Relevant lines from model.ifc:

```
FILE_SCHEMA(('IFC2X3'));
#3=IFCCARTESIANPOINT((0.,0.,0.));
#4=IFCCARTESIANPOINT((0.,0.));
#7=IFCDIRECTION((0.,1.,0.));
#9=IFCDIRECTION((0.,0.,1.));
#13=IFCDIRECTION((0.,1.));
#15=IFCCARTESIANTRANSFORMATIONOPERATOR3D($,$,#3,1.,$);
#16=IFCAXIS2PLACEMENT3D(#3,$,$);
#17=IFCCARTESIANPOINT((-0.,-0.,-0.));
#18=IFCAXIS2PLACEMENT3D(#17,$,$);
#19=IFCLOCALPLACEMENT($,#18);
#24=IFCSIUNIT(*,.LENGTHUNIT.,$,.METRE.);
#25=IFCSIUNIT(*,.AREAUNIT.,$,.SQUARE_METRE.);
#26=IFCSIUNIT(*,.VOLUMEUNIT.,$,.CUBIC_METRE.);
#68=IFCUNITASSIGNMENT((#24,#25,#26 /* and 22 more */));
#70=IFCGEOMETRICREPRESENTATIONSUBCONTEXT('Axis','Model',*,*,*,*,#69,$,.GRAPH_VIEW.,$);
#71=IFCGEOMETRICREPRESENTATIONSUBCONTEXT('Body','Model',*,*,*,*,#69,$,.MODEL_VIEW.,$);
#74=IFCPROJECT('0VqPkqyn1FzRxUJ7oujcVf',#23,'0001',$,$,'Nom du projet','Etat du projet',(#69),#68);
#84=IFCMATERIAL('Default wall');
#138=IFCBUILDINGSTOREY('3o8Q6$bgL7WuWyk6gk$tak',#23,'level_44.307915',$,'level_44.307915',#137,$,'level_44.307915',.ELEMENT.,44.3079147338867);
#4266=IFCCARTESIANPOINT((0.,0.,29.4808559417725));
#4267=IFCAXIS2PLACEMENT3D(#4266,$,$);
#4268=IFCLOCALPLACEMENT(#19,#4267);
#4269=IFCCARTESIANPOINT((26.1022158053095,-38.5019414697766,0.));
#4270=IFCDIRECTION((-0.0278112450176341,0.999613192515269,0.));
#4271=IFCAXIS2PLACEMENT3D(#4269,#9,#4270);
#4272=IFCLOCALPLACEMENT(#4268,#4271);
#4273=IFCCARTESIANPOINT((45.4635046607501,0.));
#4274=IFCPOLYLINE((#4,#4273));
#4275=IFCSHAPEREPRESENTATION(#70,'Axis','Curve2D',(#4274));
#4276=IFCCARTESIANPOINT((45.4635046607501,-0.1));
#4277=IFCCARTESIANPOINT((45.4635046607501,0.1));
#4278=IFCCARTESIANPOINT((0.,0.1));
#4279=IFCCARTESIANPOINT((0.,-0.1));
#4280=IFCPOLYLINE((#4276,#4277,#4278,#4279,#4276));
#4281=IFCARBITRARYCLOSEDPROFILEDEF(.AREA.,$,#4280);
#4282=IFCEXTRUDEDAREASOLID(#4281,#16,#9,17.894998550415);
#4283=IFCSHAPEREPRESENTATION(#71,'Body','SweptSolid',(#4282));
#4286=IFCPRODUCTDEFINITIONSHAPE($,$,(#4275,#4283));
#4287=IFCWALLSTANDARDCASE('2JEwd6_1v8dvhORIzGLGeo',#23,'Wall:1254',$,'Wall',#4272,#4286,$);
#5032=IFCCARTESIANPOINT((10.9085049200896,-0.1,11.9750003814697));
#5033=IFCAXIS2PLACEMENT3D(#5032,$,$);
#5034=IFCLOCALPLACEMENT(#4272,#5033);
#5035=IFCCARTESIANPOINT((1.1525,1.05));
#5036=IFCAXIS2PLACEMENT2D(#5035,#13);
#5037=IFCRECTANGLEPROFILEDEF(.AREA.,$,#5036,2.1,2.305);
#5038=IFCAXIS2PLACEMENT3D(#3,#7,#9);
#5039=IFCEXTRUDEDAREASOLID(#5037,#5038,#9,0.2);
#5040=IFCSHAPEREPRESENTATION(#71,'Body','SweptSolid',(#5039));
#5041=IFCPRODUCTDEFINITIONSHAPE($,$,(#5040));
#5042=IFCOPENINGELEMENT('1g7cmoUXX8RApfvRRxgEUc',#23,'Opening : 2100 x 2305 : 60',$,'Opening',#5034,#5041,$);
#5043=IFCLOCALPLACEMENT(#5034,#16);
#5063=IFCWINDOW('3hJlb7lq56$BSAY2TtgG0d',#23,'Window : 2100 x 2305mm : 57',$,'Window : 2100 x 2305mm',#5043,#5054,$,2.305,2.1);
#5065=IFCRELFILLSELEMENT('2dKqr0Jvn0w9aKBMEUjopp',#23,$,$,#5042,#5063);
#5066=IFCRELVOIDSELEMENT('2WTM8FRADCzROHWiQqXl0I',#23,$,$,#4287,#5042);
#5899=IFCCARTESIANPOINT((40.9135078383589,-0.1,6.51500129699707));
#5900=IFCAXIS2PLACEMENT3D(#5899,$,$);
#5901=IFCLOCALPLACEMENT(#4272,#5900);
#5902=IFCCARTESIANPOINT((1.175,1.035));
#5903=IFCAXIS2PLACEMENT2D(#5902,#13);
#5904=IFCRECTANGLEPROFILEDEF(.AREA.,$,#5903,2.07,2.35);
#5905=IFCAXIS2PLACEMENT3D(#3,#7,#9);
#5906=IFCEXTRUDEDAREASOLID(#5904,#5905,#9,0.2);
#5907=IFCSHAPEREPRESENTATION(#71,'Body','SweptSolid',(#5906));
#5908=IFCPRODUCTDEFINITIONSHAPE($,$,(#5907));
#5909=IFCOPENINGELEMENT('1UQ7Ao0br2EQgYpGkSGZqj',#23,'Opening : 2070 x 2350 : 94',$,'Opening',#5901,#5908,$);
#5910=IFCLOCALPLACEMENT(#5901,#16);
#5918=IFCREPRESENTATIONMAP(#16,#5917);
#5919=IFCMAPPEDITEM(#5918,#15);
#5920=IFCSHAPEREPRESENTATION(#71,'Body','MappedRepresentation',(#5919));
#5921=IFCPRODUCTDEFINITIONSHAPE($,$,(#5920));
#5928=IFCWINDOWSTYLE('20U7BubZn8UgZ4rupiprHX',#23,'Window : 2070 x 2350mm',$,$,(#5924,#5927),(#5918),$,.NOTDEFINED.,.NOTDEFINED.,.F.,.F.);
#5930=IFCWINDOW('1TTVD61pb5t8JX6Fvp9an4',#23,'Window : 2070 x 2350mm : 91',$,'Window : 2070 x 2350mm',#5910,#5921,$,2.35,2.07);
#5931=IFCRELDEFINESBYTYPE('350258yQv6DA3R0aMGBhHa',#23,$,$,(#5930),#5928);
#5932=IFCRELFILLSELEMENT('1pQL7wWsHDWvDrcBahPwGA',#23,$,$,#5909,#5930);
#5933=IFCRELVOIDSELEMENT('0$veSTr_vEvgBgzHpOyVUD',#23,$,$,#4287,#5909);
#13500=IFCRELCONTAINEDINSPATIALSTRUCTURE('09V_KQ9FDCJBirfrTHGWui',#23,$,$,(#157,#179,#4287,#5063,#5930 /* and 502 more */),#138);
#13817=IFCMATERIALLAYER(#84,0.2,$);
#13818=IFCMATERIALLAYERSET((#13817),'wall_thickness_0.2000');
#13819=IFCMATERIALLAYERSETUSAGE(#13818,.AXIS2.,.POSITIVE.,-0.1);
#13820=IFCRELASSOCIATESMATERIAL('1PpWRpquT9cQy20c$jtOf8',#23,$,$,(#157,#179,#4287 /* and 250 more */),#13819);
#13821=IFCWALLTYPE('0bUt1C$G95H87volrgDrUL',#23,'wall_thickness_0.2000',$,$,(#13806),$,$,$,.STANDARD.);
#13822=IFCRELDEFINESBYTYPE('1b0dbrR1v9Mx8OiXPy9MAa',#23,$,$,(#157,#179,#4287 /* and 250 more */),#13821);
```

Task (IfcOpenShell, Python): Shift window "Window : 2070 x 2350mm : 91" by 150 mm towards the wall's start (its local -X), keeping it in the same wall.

```python
import ifcopenshell
import ifcopenshell.api.geometry
import ifcopenshell.util.placement
import ifcopenshell.util.unit

model = ifcopenshell.open("model.ifc")
unit_scale = ifcopenshell.util.unit.calculate_unit_scale(model)

window = model.by_guid("1TTVD61pb5t8JX6Fvp9an4")
opening = window.FillsVoids[0].RelatingOpeningElement
wall = opening.VoidsElements[0].RelatingBuildingElement

wall_matrix = ifcopenshell.util.placement.get_local_placement(wall.ObjectPlacement)
shift = wall_matrix[:3, 0] * -0.15 / unit_scale
before = ifcopenshell.util.placement.get_local_placement(window.ObjectPlacement)[:3, 3].copy()

# The window is placed relative to its opening, so it follows when the opening moves.
matrix = ifcopenshell.util.placement.get_local_placement(opening.ObjectPlacement)
matrix[:3, 3] += shift
ifcopenshell.api.geometry.edit_object_placement(
    model, product=opening, matrix=matrix, is_si=False, should_transform_children=True
)

after = ifcopenshell.util.placement.get_local_placement(window.ObjectPlacement)[:3, 3]
print("window moved by", (after - before).round(3) + 0.0)

model.write("model_v2.ifc")
```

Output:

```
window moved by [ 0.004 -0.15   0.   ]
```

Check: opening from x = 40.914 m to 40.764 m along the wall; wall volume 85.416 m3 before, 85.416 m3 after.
